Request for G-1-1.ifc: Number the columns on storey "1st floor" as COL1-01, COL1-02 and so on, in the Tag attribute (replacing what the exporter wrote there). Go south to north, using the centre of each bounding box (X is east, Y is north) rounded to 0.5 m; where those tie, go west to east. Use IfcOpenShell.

First a look at what the model holds.

```python
import ifcopenshell
import ifcopenshell.util.element
import ifcopenshell.util.placement

model = ifcopenshell.open("G-1-1.ifc")
print(model.schema)
storey = next(s for s in model.by_type("IfcBuildingStorey") if s.Name == "1st floor")
columns = [e for e in ifcopenshell.util.element.get_decomposition(storey) if e.is_a("IfcColumn")]
for e in sorted(columns, key=lambda e: e.id()):
    origin = ifcopenshell.util.placement.get_local_placement(e.ObjectPlacement)[:3, 3]
    print(e.id(), e.Tag, e.Name, origin.round(2) + 0.0, sep=" | ")
```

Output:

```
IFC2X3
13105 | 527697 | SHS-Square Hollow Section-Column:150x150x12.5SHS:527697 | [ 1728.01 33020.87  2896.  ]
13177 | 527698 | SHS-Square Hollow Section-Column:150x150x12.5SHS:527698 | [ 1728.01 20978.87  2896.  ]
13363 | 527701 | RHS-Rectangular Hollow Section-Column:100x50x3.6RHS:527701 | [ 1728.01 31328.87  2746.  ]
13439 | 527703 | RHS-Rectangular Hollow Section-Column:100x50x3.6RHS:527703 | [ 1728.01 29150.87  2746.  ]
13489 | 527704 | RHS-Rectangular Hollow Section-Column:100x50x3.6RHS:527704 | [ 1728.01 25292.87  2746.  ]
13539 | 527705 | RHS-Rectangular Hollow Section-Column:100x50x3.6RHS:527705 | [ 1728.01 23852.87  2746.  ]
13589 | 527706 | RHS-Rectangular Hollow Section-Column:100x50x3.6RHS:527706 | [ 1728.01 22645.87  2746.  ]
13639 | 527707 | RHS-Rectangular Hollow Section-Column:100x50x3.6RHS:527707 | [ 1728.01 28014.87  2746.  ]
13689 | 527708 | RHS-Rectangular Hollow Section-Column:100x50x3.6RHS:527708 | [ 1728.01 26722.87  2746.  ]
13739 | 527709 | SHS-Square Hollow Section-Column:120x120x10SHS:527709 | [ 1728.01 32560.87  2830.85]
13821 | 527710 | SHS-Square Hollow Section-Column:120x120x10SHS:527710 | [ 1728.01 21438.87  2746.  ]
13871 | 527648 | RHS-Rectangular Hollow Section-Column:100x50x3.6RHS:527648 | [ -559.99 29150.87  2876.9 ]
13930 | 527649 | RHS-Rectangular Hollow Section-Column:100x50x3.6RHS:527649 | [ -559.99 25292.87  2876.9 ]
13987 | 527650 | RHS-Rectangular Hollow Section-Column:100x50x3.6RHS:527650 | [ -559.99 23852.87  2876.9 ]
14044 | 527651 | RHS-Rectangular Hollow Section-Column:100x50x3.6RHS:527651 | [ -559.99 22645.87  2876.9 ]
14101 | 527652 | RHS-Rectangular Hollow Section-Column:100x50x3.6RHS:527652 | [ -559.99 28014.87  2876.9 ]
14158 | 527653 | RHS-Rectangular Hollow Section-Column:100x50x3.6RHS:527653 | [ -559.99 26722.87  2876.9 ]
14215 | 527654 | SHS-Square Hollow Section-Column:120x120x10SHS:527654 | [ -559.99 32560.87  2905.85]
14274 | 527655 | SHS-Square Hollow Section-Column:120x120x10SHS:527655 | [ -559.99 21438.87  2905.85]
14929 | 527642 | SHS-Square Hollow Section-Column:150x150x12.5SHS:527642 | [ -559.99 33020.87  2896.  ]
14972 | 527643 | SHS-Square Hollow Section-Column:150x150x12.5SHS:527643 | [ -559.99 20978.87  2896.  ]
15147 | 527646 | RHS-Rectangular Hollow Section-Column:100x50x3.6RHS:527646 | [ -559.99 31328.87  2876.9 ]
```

```python
import ifcopenshell
import ifcopenshell.geom
import ifcopenshell.util.element
import ifcopenshell.util.shape

model = ifcopenshell.open("G-1-1.ifc")
settings = ifcopenshell.geom.settings()
settings.set("use-world-coords", True)


def centre(element):
    shape = ifcopenshell.geom.create_shape(settings, element)
    return ifcopenshell.util.shape.get_bbox_centroid(shape.geometry)


storey = next(s for s in model.by_type("IfcBuildingStorey") if s.Name == "1st floor")
columns = [e for e in ifcopenshell.util.element.get_decomposition(storey) if e.is_a("IfcColumn")]

# Insertion points can sit at a corner or the storey origin, so sort by the geometry (in metres).
centres = {e: centre(e) for e in columns}
columns.sort(key=lambda e: (round(centres[e][1] / 0.5), centres[e][0]))

for i, e in enumerate(columns, start=1):
    number = f"COL1-{i:02d}"
    e.Tag = number
    print(e.id(), number)

model.write("G-1-1_edited.ifc")
```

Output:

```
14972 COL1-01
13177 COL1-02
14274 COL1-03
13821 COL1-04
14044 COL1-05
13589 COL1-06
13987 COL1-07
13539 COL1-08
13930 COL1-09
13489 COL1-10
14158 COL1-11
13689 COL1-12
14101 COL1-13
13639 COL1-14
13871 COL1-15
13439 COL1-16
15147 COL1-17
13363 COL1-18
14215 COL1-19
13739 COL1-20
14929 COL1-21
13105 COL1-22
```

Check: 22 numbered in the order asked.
